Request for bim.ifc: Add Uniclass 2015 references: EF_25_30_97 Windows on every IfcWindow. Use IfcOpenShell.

First a look at what the model holds.

```python
import ifcopenshell

model = ifcopenshell.open("bim.ifc")
print(model.schema)
print("classifications:", [c.Name for c in model.by_type("IfcClassification")])
for ifc_class in ("IfcDoor", "IfcRoof", "IfcStair", "IfcWall", "IfcWindow"):
    print(ifc_class, len(model.by_type(ifc_class)))
```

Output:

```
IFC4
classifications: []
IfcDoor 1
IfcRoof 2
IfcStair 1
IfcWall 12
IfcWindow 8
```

```python
import ifcopenshell
import ifcopenshell.api.classification

model = ifcopenshell.open("bim.ifc")

system = ifcopenshell.api.classification.add_classification(model, classification="Uniclass 2015")

codes = {
    "IfcWindow": ("EF_25_30_97", "Windows"),
}
for ifc_class, (code, name) in codes.items():
    products = model.by_type(ifc_class)
    ifcopenshell.api.classification.add_reference(
        model, products=products, classification=system, identification=code, name=name
    )
    print(code, len(products))

model.write("bim_rev.ifc")
```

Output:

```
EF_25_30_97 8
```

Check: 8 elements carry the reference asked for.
